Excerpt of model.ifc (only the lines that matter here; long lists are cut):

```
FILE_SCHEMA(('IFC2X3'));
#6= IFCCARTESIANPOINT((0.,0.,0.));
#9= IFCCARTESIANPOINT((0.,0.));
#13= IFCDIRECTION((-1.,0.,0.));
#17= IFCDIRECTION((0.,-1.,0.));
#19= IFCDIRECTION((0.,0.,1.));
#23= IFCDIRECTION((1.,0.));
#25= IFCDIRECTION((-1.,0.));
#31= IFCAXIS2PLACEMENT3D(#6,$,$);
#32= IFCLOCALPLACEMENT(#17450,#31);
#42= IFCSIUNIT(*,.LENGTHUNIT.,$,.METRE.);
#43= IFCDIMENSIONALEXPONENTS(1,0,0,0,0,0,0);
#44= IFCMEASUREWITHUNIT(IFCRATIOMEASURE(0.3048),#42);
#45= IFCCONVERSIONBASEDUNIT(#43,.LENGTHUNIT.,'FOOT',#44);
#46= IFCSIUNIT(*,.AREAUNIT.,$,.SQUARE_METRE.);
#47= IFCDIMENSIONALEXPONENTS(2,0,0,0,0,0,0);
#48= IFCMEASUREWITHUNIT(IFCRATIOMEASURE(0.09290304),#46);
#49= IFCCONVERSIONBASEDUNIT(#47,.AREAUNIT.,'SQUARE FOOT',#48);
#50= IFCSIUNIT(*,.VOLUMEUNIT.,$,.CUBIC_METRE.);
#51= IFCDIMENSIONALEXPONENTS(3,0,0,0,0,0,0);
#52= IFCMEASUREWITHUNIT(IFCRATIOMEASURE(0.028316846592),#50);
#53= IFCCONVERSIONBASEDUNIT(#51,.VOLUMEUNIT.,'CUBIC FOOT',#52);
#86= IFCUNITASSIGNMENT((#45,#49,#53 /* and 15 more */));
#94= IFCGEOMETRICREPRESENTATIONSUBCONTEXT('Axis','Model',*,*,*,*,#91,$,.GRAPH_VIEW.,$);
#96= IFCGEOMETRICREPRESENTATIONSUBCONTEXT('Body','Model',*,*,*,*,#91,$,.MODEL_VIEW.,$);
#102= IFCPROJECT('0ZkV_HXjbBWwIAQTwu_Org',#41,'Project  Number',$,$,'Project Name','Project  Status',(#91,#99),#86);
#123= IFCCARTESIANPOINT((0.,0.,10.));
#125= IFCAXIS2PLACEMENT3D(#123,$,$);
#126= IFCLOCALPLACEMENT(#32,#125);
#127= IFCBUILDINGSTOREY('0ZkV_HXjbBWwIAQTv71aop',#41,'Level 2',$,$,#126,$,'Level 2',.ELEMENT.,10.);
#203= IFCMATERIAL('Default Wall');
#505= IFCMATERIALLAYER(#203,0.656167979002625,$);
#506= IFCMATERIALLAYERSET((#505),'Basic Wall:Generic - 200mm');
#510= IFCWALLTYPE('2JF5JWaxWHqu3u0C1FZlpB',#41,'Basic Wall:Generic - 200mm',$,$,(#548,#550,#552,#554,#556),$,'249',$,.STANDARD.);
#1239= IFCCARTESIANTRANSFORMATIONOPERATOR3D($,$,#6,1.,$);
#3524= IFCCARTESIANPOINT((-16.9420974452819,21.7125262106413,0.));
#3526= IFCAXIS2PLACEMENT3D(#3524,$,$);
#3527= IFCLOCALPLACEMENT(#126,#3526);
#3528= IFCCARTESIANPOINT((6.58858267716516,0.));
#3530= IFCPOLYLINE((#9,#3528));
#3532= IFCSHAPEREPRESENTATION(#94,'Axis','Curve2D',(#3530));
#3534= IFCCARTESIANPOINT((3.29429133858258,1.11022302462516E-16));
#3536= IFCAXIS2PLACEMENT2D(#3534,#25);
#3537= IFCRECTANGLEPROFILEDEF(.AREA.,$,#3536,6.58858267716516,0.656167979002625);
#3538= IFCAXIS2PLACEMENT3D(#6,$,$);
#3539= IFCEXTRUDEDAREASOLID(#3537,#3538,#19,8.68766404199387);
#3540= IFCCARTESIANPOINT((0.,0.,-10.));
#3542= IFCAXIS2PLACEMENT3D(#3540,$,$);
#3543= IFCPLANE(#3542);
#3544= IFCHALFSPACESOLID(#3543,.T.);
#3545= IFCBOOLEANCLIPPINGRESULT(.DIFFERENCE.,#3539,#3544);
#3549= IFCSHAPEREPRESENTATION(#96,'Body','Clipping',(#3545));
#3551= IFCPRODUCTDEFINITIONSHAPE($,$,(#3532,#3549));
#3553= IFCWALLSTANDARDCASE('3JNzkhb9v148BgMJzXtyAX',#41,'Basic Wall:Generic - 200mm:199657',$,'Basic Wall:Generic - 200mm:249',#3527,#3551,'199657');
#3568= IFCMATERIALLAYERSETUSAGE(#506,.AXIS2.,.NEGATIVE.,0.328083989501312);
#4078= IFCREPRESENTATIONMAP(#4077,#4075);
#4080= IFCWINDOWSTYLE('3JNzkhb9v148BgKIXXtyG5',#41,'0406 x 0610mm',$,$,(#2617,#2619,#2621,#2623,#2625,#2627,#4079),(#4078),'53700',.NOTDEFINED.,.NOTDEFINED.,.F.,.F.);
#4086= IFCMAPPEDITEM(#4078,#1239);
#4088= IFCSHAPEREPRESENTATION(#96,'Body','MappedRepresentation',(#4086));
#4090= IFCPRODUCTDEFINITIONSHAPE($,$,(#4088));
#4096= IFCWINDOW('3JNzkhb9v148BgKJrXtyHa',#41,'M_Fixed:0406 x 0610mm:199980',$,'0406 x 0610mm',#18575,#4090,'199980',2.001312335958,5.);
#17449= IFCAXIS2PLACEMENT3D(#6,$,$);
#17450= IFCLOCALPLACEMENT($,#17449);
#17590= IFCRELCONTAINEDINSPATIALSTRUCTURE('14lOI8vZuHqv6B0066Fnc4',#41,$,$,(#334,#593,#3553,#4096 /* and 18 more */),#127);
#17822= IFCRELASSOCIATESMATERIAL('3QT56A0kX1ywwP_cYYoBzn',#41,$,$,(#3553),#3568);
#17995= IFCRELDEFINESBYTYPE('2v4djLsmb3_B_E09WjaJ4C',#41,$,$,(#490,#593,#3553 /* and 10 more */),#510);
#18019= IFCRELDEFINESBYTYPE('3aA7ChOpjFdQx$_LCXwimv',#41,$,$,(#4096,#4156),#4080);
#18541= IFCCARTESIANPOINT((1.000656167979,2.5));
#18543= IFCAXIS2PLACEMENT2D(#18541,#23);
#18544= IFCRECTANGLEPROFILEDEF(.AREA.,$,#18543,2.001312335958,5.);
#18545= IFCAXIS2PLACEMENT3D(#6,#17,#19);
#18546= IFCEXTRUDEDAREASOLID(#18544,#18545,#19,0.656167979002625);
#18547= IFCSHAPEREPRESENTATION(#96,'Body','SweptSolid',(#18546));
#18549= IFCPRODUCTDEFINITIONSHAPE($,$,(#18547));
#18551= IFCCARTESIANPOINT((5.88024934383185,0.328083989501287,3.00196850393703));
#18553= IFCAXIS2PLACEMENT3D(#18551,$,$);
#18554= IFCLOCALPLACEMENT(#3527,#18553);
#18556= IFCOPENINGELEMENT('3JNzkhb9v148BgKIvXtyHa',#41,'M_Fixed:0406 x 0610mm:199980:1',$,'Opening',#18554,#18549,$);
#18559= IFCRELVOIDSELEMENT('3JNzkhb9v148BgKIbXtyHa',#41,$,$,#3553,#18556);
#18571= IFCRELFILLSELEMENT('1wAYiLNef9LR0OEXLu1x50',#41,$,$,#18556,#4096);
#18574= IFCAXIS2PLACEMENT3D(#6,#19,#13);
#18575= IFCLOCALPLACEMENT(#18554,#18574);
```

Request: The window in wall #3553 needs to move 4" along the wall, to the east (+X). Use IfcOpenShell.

```python
import ifcopenshell
import ifcopenshell.api.geometry
import ifcopenshell.util.placement
import ifcopenshell.util.unit

model = ifcopenshell.open("model.ifc")
unit_scale = ifcopenshell.util.unit.calculate_unit_scale(model)

window = model.by_guid("3JNzkhb9v148BgKJrXtyHa")
opening = window.FillsVoids[0].RelatingOpeningElement
wall = opening.VoidsElements[0].RelatingBuildingElement

wall_matrix = ifcopenshell.util.placement.get_local_placement(wall.ObjectPlacement)
shift = wall_matrix[:3, 0] * 4 * 0.0254 / unit_scale
before = ifcopenshell.util.placement.get_local_placement(window.ObjectPlacement)[:3, 3].copy()

# The window is placed relative to its opening, so it follows when the opening moves.
matrix = ifcopenshell.util.placement.get_local_placement(opening.ObjectPlacement)
matrix[:3, 3] += shift
ifcopenshell.api.geometry.edit_object_placement(
    model, product=opening, matrix=matrix, is_si=False, should_transform_children=True
)

after = ifcopenshell.util.placement.get_local_placement(window.ObjectPlacement)[:3, 3]
print("window moved by", (after - before).round(3) + 0.0)

model.write("model-out.ifc")
```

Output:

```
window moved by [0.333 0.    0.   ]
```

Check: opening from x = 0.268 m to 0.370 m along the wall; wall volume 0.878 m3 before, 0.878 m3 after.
